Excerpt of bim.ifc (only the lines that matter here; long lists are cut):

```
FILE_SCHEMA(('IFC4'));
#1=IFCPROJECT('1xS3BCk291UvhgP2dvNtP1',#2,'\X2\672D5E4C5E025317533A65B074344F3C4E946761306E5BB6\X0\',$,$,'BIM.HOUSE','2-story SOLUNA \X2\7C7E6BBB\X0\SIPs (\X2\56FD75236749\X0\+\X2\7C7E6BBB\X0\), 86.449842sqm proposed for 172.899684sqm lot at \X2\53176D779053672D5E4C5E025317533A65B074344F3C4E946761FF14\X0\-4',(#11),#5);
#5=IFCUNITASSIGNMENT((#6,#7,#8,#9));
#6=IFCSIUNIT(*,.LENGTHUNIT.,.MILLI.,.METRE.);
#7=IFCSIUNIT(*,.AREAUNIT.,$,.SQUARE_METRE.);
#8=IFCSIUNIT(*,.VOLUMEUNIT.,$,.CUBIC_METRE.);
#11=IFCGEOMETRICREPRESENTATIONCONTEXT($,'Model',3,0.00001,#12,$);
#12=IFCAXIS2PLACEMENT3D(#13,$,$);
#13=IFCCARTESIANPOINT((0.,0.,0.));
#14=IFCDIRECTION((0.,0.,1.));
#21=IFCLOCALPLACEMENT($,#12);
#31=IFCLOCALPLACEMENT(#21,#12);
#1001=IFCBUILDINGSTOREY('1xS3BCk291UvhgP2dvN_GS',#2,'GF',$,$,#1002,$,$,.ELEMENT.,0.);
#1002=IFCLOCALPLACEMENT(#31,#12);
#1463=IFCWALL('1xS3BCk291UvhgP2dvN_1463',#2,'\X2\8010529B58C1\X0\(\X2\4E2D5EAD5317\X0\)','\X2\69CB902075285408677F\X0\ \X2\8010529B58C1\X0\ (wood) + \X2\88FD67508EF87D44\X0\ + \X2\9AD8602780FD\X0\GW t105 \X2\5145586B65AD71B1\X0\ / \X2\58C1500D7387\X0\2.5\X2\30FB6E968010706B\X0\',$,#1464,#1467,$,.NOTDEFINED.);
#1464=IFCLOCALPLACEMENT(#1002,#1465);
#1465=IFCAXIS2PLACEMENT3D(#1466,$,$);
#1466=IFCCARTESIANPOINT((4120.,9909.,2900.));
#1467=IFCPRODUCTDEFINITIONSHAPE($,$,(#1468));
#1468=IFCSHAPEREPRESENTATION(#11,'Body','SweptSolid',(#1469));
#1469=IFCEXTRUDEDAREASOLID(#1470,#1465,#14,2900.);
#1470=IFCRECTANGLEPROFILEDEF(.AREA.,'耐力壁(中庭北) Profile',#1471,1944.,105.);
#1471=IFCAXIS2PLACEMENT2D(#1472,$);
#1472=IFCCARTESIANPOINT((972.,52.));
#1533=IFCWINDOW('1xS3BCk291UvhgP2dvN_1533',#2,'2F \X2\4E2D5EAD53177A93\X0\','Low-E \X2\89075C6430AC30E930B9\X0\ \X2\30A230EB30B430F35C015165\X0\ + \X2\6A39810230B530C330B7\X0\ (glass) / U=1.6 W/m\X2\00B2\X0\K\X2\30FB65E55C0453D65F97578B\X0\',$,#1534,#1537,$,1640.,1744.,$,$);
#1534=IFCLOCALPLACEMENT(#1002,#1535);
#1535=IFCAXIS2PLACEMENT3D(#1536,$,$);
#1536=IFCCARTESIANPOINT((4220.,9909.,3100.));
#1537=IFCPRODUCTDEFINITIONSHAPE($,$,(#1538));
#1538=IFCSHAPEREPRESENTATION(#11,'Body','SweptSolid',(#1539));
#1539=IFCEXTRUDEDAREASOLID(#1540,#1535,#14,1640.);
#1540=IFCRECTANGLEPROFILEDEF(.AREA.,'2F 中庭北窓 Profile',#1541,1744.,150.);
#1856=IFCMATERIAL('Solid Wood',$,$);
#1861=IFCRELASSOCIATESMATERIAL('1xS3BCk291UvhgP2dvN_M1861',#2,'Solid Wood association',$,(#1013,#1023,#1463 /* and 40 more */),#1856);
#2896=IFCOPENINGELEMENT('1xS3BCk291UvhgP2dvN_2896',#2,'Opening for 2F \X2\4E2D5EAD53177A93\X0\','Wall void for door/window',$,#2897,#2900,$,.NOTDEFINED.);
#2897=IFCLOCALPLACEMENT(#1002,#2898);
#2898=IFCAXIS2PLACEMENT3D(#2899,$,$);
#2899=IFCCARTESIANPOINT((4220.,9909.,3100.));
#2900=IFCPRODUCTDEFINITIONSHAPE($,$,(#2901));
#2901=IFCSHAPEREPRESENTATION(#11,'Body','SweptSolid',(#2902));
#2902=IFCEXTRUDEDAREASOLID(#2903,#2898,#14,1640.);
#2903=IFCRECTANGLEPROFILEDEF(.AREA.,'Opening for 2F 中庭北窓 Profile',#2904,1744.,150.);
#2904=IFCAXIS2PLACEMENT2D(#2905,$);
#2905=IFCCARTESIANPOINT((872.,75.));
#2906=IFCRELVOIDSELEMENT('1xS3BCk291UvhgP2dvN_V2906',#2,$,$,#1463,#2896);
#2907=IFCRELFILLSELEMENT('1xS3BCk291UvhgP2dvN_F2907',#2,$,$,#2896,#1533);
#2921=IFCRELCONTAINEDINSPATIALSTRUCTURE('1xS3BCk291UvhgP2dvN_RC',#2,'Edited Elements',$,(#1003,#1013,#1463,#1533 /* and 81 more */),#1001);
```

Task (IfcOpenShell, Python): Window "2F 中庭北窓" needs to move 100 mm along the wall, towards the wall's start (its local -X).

```python
import ifcopenshell
import ifcopenshell.api.geometry
import ifcopenshell.util.placement
import ifcopenshell.util.unit

model = ifcopenshell.open("bim.ifc")
unit_scale = ifcopenshell.util.unit.calculate_unit_scale(model)

window = model.by_guid("1xS3BCk291UvhgP2dvN_1533")
opening = window.FillsVoids[0].RelatingOpeningElement
wall = opening.VoidsElements[0].RelatingBuildingElement

wall_matrix = ifcopenshell.util.placement.get_local_placement(wall.ObjectPlacement)
shift = wall_matrix[:3, 0] * -0.1 / unit_scale
before = ifcopenshell.util.placement.get_local_placement(window.ObjectPlacement)[:3, 3].copy()

# The window is not placed relative to its opening, so move both.
for product in (opening, window):
    matrix = ifcopenshell.util.placement.get_local_placement(product.ObjectPlacement)
    matrix[:3, 3] += shift
    ifcopenshell.api.geometry.edit_object_placement(model, product=product, matrix=matrix, is_si=False)

after = ifcopenshell.util.placement.get_local_placement(window.ObjectPlacement)[:3, 3]
print("window moved by", (after - before).round(3) + 0.0)

model.write("bim_rev.ifc")
```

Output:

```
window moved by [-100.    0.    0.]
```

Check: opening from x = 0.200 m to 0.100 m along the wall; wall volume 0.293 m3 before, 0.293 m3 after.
